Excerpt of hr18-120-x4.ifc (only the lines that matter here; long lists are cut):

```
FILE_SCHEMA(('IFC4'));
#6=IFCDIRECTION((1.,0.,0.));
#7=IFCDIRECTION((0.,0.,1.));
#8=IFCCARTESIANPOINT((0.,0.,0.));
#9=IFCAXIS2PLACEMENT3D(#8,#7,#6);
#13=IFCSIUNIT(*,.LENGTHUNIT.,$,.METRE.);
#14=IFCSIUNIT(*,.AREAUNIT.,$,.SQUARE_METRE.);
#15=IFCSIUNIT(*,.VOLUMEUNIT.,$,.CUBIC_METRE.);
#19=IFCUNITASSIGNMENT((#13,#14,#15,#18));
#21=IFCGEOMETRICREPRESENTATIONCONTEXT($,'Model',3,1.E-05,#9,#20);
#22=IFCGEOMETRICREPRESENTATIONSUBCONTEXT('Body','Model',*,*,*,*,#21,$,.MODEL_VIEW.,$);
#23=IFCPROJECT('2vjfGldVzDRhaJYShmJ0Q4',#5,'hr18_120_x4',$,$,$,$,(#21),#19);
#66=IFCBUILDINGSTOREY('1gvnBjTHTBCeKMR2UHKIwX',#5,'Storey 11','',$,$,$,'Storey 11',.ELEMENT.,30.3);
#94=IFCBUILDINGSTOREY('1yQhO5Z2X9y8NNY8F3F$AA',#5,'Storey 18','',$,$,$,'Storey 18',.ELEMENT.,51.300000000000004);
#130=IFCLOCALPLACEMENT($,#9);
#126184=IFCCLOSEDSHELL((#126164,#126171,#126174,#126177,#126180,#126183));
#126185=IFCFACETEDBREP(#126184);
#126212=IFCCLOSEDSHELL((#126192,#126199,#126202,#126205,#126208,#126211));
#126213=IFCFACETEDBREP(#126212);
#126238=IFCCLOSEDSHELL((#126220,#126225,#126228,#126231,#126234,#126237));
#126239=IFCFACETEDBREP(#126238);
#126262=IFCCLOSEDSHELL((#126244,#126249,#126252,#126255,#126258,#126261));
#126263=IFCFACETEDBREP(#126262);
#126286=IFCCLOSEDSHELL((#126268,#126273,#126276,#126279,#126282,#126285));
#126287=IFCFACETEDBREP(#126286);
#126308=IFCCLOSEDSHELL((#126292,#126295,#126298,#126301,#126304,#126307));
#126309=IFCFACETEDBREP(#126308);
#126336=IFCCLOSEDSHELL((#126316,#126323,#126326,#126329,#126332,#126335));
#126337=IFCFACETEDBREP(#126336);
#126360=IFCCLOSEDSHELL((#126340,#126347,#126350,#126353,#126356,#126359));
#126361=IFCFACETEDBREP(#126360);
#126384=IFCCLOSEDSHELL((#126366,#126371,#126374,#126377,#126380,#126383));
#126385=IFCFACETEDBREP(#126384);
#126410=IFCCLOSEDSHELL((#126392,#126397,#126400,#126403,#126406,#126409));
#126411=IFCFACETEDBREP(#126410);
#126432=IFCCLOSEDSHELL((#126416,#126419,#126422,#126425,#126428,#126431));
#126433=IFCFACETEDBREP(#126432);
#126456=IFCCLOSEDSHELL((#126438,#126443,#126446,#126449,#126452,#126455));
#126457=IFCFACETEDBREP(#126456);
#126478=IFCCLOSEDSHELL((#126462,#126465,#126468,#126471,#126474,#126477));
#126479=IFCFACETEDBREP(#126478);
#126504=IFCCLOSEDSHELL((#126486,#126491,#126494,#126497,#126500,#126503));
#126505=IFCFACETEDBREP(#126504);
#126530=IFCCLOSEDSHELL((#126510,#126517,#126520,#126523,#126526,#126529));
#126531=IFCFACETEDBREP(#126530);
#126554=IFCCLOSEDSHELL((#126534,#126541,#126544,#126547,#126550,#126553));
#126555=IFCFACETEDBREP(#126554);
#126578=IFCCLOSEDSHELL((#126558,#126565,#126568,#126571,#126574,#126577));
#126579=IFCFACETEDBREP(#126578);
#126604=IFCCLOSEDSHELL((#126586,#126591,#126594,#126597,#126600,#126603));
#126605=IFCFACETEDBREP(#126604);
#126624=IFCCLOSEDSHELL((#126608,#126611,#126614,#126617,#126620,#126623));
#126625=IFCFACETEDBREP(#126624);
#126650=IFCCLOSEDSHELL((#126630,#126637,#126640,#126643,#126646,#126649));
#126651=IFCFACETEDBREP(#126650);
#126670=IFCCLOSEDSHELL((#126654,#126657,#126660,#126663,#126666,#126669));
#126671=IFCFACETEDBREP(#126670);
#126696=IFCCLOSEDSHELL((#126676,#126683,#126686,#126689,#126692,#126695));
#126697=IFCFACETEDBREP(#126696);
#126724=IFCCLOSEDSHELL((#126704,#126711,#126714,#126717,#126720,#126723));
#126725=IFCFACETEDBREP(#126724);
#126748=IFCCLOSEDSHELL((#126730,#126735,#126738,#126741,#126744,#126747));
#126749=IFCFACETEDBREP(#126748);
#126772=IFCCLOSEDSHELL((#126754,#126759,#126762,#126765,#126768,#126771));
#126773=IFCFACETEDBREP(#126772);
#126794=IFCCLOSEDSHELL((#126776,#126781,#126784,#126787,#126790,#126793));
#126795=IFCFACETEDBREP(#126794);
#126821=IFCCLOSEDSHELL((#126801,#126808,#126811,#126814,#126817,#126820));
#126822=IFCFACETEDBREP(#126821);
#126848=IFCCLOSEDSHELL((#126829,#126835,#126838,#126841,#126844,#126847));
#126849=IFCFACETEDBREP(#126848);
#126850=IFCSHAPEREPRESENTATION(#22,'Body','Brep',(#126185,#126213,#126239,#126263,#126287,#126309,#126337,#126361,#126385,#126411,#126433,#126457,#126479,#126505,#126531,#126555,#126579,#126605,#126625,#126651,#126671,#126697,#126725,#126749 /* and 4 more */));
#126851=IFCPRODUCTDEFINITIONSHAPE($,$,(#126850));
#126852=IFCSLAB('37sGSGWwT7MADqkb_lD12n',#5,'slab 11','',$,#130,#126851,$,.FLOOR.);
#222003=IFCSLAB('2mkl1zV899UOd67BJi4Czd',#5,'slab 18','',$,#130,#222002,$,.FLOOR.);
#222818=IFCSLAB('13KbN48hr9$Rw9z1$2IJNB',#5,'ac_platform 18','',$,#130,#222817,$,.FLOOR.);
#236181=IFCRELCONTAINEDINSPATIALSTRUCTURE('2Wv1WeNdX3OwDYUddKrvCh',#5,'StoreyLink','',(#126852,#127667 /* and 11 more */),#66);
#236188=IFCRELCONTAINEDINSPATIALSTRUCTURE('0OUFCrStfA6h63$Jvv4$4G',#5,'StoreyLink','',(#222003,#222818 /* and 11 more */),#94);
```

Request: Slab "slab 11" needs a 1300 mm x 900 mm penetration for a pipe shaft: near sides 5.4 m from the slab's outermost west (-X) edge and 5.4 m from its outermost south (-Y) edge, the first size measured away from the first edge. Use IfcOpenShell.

```python
import numpy as np
import ifcopenshell
import ifcopenshell.api.feature
import ifcopenshell.api.geometry
import ifcopenshell.api.root
import ifcopenshell.geom
import ifcopenshell.util.placement
import ifcopenshell.util.representation
import ifcopenshell.util.shape
import ifcopenshell.util.unit

model = ifcopenshell.open("hr18-120-x4.ifc")
unit_scale = ifcopenshell.util.unit.calculate_unit_scale(model)
settings = ifcopenshell.geom.settings()


def volume(element):
    """Net volume in cubic metres, openings subtracted."""
    shape = ifcopenshell.geom.create_shape(settings, element)
    return ifcopenshell.util.shape.get_volume(shape.geometry)


slab = model.by_guid("37sGSGWwT7MADqkb_lD12n")
before = volume(slab)

# Extent in the slab's own axes, in metres. The edges named are its -X and -Y sides.
slab_shape = ifcopenshell.geom.create_shape(settings, slab)
vertices = ifcopenshell.util.shape.get_vertices(slab_shape.geometry)
x_min, y_min, bottom = vertices.min(axis=0)
top = vertices[:, 2].max()

opening = ifcopenshell.api.root.create_entity(model, ifc_class="IfcOpeningElement", name="Pipe shaft opening", predefined_type="OPENING")
context = ifcopenshell.util.representation.get_context(model, "Model", "Body", "MODEL_VIEW")
width, depth = 1.3, 0.9
outline = [(0.0, 0.0), (width, 0.0), (width, depth), (0.0, depth), (0.0, 0.0)]
# Overshoot both faces by 50 mm so the cut is clean.
shape = ifcopenshell.api.geometry.add_slab_representation(
    model, context=context, depth=top - bottom + 0.1, polyline=outline
)
ifcopenshell.api.geometry.assign_representation(model, product=opening, representation=shape)

matrix = ifcopenshell.util.placement.get_local_placement(slab.ObjectPlacement)
matrix[:, 3] = matrix @ np.append(np.array([x_min + 5.4, y_min + 5.4, bottom - 0.05]) / unit_scale, 1.0)
ifcopenshell.api.geometry.edit_object_placement(model, product=opening, matrix=matrix, is_si=False)
ifcopenshell.api.feature.add_feature(model, feature=opening, element=slab)

after = volume(slab)

print(f"slab volume {before:.3f} -> {after:.3f} m3")

model.write("hr18-120-x4_rev.ifc")
```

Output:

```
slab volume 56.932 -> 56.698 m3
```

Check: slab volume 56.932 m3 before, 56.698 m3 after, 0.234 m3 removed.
